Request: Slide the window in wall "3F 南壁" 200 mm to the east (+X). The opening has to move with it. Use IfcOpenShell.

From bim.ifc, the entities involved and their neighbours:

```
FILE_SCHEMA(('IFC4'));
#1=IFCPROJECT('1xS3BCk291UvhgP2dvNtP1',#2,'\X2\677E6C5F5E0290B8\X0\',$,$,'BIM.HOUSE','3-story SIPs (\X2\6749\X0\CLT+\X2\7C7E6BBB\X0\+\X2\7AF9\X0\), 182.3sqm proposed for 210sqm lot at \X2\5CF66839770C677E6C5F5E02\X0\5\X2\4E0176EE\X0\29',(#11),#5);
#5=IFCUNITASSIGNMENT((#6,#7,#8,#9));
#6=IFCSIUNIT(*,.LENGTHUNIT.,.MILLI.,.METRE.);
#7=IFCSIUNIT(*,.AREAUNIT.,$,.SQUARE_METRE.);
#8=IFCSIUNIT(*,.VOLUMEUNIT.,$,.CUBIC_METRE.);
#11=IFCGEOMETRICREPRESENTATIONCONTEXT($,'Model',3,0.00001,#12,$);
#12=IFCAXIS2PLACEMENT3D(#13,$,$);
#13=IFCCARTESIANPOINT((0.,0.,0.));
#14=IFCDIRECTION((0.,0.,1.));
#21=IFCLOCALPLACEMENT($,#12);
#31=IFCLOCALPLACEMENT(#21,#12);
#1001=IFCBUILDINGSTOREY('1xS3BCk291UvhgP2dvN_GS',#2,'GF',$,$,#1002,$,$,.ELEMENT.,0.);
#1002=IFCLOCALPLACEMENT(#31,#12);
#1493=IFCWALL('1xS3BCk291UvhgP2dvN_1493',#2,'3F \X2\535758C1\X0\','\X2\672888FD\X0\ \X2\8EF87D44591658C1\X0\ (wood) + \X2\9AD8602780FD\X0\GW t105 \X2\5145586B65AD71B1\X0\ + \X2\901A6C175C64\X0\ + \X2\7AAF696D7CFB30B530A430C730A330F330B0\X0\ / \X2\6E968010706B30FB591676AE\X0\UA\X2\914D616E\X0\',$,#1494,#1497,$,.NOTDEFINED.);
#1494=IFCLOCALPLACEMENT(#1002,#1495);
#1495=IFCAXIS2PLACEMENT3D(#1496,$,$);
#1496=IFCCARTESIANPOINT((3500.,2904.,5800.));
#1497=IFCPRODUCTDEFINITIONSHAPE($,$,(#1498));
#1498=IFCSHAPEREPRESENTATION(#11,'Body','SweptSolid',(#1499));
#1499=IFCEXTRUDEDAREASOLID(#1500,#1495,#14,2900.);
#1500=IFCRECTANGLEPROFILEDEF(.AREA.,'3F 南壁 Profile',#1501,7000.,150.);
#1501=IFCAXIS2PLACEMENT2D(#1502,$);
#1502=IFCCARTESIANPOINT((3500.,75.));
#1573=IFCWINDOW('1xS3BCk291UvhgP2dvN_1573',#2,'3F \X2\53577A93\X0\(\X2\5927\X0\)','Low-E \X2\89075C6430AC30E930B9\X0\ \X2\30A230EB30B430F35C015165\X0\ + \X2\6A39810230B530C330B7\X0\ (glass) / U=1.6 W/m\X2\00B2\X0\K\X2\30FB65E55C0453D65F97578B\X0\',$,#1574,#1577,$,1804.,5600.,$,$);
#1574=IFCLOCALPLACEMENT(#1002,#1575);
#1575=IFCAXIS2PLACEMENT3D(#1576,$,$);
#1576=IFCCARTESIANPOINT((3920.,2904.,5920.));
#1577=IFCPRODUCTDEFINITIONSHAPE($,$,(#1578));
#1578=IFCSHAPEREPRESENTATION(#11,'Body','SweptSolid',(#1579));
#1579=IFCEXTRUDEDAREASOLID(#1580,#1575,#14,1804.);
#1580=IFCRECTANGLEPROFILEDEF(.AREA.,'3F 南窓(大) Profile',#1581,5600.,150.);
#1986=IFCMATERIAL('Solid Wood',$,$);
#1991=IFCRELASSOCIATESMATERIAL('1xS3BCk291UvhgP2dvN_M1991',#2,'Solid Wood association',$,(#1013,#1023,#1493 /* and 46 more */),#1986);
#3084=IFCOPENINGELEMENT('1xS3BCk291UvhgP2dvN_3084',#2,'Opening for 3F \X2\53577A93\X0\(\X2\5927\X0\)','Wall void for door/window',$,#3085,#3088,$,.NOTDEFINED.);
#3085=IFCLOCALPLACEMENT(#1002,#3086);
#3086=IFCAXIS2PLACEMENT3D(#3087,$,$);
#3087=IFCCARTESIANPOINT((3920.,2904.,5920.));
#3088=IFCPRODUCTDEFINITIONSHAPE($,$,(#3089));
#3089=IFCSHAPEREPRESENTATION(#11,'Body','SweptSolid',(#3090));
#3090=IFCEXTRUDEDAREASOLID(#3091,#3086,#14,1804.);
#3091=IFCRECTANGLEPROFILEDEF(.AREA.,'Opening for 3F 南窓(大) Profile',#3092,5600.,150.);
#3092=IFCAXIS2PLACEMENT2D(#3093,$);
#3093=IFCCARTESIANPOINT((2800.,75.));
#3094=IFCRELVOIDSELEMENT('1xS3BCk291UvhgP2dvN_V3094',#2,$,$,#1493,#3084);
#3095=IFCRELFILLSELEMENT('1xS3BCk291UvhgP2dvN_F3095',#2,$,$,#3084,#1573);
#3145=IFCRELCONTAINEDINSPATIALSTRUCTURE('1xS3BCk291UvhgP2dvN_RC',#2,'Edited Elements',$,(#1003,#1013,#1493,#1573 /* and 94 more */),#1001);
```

```python
import ifcopenshell
import ifcopenshell.api.geometry
import ifcopenshell.util.placement

model = ifcopenshell.open("bim.ifc")

window = model.by_guid("1xS3BCk291UvhgP2dvN_1573")
opening = window.FillsVoids[0].RelatingOpeningElement
wall = opening.VoidsElements[0].RelatingBuildingElement

wall_matrix = ifcopenshell.util.placement.get_local_placement(wall.ObjectPlacement)
shift = wall_matrix[:3, 0] * 200.0
before = ifcopenshell.util.placement.get_local_placement(window.ObjectPlacement)[:3, 3].copy()

# The window is not placed relative to its opening, so move both.
for product in (opening, window):
    matrix = ifcopenshell.util.placement.get_local_placement(product.ObjectPlacement)
    matrix[:3, 3] += shift
    ifcopenshell.api.geometry.edit_object_placement(model, product=product, matrix=matrix, is_si=False)

after = ifcopenshell.util.placement.get_local_placement(window.ObjectPlacement)[:3, 3]
print("window moved by", (after - before).round(3) + 0.0)

model.write("bim_updated.ifc")
```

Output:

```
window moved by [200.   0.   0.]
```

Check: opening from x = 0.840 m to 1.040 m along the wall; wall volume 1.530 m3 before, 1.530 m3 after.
